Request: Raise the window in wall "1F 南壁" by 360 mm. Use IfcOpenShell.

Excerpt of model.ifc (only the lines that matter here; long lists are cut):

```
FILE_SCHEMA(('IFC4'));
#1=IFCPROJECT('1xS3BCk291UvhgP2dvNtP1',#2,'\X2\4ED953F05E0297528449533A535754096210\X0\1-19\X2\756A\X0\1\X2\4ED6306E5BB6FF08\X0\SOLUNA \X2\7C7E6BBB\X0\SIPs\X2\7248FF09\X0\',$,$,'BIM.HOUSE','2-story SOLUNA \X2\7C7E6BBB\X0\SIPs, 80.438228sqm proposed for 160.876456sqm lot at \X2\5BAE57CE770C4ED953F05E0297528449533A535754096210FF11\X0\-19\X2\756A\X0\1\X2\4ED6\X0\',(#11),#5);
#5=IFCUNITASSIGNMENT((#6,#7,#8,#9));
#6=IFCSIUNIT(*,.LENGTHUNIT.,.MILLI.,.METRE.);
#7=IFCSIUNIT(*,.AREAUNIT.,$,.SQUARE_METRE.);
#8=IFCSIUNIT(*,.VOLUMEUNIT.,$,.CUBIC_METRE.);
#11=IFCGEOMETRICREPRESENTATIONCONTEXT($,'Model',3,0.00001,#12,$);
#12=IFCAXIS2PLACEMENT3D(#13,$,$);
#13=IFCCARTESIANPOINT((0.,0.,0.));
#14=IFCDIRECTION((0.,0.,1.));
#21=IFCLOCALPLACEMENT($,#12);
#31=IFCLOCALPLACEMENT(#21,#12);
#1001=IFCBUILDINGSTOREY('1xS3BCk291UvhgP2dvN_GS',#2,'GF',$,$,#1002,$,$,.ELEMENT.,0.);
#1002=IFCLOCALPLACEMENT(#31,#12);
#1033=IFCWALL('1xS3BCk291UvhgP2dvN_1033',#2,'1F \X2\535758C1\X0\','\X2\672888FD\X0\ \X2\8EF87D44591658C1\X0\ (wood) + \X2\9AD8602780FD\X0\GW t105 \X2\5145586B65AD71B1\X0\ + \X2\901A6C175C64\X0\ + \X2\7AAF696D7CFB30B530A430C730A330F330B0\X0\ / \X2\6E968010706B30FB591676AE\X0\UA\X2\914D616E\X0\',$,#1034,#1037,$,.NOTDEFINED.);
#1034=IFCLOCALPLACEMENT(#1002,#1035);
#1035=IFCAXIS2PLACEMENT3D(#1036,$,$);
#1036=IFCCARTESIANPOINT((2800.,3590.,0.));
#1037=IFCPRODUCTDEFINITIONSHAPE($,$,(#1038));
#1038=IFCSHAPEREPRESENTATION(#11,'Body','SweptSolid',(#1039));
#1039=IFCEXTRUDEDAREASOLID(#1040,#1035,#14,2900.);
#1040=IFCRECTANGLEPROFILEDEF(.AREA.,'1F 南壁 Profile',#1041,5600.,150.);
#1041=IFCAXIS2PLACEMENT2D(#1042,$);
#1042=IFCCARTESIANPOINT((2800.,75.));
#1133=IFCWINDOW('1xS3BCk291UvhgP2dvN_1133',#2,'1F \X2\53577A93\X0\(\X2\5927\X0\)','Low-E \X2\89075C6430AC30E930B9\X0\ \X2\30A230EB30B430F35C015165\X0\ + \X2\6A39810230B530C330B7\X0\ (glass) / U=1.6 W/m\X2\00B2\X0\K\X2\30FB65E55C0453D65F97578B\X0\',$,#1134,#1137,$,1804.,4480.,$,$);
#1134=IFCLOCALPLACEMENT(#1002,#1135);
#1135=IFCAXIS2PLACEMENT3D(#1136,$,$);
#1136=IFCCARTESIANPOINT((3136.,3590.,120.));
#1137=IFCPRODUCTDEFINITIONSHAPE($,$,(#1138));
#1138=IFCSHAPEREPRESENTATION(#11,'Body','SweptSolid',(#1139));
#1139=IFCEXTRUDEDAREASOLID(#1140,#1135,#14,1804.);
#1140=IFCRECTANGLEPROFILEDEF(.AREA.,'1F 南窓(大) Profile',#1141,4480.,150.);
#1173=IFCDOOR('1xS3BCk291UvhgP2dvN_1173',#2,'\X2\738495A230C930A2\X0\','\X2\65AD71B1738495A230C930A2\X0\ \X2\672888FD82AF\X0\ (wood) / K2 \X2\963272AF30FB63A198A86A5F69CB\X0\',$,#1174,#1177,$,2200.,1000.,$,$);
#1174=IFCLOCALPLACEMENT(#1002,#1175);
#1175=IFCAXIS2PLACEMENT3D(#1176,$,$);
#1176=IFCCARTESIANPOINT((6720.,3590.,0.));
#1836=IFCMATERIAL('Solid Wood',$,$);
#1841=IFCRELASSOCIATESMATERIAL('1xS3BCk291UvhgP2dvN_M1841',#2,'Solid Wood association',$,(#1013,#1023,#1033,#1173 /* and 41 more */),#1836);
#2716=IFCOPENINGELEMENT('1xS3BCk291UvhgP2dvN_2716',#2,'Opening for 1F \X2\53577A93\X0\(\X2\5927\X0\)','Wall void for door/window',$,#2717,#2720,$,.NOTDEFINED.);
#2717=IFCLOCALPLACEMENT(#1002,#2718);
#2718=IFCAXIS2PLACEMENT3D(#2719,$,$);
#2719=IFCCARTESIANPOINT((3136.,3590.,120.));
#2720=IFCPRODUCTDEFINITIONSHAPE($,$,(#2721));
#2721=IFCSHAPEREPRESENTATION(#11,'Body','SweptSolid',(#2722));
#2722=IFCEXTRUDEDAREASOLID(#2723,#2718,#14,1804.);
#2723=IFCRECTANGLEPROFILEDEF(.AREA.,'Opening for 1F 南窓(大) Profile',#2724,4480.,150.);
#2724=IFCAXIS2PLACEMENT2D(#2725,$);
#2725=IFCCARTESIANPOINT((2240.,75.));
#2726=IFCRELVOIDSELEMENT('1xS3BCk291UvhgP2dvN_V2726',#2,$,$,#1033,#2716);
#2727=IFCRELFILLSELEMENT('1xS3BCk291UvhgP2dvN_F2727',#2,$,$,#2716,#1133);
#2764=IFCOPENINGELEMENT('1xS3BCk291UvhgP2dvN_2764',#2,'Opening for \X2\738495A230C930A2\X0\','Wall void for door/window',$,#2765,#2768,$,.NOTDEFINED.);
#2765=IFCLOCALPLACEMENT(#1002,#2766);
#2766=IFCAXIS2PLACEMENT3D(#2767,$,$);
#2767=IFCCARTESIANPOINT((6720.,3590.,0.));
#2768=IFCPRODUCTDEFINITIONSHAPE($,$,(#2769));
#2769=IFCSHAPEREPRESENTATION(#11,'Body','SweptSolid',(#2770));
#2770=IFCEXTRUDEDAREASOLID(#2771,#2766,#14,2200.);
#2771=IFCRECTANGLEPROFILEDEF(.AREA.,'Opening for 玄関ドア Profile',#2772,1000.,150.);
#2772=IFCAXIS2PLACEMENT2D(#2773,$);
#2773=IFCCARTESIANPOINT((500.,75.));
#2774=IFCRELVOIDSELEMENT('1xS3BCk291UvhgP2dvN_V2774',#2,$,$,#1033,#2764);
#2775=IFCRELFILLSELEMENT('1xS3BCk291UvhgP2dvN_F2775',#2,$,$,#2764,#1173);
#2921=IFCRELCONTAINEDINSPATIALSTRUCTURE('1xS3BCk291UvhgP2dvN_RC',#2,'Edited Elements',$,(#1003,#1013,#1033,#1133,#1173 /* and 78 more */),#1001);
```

```python
import numpy as np
import ifcopenshell
import ifcopenshell.api.geometry
import ifcopenshell.util.placement
import ifcopenshell.util.unit

model = ifcopenshell.open("model.ifc")
unit_scale = ifcopenshell.util.unit.calculate_unit_scale(model)

window = model.by_guid("1xS3BCk291UvhgP2dvN_1133")
opening = window.FillsVoids[0].RelatingOpeningElement
dz = 0.36 / unit_scale

shift = np.array([0.0, 0.0, dz])
# The window is not placed relative to its opening, so move both.
for product in (opening, window):
    matrix = ifcopenshell.util.placement.get_local_placement(product.ObjectPlacement)
    matrix[:3, 3] += shift
    ifcopenshell.api.geometry.edit_object_placement(model, product=product, matrix=matrix, is_si=False)

print(f"moved by {dz * unit_scale:+.3f} m")

model.write("model-out.ifc")
```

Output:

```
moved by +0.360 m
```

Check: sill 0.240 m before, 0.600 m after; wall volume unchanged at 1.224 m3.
